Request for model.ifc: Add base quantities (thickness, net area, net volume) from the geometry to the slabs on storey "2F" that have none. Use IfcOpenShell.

First a look at what the model holds.

```python
import ifcopenshell
import ifcopenshell.util.element
import ifcopenshell.util.unit

model = ifcopenshell.open("model.ifc")
print(model.schema)
for unit_type in ("LENGTHUNIT", "AREAUNIT", "VOLUMEUNIT"):
    print(unit_type, ifcopenshell.util.unit.calculate_unit_scale(model, unit_type))
storey = next(s for s in model.by_type("IfcBuildingStorey") if s.Name == "2F")
slabs = [e for e in ifcopenshell.util.element.get_decomposition(storey) if e.is_a("IfcSlab")]
for e in sorted(slabs, key=lambda e: e.id()):
    print(e.id(), e.is_a(), e.Name, list(ifcopenshell.util.element.get_psets(e, qtos_only=True)), sep=" | ")
```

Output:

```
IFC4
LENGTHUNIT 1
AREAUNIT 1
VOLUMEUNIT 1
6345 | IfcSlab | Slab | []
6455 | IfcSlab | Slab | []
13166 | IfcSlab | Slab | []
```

```python
import ifcopenshell
import ifcopenshell.api.pset
import ifcopenshell.geom
import ifcopenshell.util.element
import ifcopenshell.util.shape
import ifcopenshell.util.unit

model = ifcopenshell.open("model.ifc")
unit_scale = ifcopenshell.util.unit.calculate_unit_scale(model)
area_scale = ifcopenshell.util.unit.calculate_unit_scale(model, "AREAUNIT")
volume_scale = ifcopenshell.util.unit.calculate_unit_scale(model, "VOLUMEUNIT")
settings = ifcopenshell.geom.settings()

storey = next(s for s in model.by_type("IfcBuildingStorey") if s.Name == "2F")
slabs = [e for e in ifcopenshell.util.element.get_decomposition(storey) if e.is_a("IfcSlab")]

for e in sorted(slabs, key=lambda e: e.id()):
    if ifcopenshell.util.element.get_psets(e, qtos_only=True, should_inherit=False):
        continue
    # Geometry comes back in metres, in the element's own axes.
    shape = ifcopenshell.geom.create_shape(settings, e)
    values = {
        "Width": ifcopenshell.util.shape.get_z(shape.geometry) / unit_scale,
        "NetArea": ifcopenshell.util.shape.get_footprint_area(shape.geometry) / area_scale,
        "NetVolume": ifcopenshell.util.shape.get_volume(shape.geometry) / volume_scale,
    }
    qto = ifcopenshell.api.pset.add_qto(model, product=e, name="Qto_SlabBaseQuantities")
    ifcopenshell.api.pset.edit_qto(model, qto=qto, properties=values)
    print(e.id(), {k: round(v, 3) for k, v in values.items()})

model.write("model-out.ifc")
```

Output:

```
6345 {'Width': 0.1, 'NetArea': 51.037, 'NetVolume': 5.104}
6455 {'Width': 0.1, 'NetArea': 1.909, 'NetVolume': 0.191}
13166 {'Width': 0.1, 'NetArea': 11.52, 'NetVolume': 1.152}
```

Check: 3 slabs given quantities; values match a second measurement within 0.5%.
